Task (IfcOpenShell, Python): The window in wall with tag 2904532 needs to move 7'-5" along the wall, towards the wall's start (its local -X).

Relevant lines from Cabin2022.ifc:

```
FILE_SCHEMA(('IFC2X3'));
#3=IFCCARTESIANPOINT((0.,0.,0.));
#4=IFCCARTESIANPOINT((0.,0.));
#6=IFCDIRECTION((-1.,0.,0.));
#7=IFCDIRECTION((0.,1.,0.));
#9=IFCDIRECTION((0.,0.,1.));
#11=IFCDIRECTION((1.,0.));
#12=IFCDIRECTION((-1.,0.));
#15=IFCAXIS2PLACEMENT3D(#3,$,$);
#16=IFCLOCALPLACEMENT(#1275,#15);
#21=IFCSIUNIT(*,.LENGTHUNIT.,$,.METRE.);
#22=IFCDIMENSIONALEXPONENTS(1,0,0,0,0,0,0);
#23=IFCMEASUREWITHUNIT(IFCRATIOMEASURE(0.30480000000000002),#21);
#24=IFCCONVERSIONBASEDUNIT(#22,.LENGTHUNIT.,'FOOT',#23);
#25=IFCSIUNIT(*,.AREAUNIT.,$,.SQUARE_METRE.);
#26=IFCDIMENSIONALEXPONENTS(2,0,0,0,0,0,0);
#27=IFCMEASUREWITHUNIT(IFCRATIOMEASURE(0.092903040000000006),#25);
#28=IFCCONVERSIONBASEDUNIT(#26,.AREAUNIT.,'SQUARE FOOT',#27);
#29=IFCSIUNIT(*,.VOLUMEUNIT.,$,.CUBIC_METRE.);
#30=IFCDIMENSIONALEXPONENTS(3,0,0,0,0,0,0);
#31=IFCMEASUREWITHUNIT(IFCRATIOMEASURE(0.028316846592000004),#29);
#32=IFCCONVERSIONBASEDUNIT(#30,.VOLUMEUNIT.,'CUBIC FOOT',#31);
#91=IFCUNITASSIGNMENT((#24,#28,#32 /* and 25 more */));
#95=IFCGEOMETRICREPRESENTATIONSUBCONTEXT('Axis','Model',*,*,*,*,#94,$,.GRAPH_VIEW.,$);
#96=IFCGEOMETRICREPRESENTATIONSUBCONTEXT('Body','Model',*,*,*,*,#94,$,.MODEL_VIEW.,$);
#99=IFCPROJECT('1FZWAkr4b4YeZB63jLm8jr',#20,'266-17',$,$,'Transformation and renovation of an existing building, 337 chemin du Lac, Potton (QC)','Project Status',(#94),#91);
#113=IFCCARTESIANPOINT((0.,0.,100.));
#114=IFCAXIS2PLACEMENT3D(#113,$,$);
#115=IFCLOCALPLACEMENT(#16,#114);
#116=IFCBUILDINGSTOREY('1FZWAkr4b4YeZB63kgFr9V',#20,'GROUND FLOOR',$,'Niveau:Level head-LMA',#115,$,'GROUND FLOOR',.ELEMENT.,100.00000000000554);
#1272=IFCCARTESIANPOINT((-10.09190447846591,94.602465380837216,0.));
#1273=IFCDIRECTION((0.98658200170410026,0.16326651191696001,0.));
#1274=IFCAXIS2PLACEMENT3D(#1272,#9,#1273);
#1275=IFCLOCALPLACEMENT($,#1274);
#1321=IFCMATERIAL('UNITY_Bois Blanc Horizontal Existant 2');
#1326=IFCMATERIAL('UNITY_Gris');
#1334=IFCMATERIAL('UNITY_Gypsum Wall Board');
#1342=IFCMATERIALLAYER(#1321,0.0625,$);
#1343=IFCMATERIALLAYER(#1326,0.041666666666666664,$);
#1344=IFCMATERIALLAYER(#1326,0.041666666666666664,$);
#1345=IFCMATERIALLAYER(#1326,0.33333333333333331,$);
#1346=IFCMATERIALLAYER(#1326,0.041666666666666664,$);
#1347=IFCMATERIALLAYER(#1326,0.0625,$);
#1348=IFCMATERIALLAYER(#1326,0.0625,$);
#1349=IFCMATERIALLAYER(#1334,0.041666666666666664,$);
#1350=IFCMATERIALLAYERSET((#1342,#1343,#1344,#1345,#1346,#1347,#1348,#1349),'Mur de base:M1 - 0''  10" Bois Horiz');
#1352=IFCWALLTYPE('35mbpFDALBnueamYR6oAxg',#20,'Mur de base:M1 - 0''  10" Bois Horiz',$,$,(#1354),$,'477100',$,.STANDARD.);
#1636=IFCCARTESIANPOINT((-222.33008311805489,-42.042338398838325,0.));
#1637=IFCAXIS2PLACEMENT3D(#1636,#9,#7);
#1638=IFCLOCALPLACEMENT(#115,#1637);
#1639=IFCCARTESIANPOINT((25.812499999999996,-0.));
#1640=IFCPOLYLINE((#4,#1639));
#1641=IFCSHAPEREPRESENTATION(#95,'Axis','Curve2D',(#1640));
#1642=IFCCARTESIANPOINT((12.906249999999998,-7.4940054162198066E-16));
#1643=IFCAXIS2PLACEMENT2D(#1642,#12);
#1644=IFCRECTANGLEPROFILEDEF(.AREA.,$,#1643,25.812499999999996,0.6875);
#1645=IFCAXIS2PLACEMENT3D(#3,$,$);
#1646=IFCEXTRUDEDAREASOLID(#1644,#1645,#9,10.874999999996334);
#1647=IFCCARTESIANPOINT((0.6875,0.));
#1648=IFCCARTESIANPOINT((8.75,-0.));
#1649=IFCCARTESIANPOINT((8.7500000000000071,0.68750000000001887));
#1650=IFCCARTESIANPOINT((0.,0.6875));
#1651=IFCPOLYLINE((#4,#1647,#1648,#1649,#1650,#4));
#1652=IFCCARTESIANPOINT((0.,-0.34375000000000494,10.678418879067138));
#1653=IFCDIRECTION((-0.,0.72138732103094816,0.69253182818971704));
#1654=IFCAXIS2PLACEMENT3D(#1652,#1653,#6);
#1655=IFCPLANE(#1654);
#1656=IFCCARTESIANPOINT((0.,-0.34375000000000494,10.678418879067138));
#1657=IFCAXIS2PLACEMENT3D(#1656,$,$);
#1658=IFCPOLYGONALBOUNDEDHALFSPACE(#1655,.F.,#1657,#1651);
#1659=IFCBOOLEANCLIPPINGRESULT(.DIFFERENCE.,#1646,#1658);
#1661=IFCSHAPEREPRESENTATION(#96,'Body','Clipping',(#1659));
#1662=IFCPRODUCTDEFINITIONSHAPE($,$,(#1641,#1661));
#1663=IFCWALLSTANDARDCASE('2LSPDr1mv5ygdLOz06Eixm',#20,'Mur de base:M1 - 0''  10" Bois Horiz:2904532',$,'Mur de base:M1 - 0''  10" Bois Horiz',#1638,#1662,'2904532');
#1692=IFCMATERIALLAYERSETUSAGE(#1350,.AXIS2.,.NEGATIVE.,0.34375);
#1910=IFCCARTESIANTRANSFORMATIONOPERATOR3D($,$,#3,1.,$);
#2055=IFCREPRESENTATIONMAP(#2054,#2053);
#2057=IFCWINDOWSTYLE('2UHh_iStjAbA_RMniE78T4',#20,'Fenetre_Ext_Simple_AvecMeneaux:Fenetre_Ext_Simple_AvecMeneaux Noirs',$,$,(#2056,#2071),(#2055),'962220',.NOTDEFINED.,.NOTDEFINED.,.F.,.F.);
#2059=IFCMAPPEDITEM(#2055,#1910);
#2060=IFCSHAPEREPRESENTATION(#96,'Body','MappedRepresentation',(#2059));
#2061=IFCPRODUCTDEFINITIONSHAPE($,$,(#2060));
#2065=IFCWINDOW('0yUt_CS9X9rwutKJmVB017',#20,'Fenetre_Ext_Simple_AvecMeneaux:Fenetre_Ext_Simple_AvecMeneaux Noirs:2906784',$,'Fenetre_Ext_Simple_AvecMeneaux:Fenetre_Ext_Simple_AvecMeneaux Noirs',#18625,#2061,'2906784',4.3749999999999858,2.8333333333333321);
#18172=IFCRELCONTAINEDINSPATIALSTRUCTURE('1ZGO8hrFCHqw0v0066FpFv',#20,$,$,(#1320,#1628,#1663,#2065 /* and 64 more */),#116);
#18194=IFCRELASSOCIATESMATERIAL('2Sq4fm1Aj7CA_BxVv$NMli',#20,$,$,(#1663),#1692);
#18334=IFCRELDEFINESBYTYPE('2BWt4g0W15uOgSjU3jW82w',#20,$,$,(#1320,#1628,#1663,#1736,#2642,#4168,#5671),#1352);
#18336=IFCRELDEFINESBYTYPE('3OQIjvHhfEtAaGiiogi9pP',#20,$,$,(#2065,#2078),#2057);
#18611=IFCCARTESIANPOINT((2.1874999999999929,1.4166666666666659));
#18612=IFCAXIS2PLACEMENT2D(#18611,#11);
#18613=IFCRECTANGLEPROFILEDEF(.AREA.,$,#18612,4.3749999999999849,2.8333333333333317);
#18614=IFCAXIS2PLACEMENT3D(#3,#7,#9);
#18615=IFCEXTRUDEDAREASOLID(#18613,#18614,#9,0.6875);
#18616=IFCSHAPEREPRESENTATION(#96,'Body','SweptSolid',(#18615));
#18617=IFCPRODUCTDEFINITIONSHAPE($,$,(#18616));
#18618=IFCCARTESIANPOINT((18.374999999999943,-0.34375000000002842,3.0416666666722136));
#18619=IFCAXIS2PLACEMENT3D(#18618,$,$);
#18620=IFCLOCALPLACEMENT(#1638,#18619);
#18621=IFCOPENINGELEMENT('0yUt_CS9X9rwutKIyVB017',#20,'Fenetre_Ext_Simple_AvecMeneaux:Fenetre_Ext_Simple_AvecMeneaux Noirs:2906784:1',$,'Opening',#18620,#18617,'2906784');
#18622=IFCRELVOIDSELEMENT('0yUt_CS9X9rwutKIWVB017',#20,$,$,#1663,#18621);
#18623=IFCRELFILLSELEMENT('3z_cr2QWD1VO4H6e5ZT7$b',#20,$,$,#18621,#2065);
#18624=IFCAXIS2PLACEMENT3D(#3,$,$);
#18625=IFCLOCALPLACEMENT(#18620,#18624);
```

```python
import ifcopenshell
import ifcopenshell.api.geometry
import ifcopenshell.util.placement
import ifcopenshell.util.unit

model = ifcopenshell.open("Cabin2022.ifc")
unit_scale = ifcopenshell.util.unit.calculate_unit_scale(model)

window = model.by_guid("0yUt_CS9X9rwutKJmVB017")
opening = window.FillsVoids[0].RelatingOpeningElement
wall = opening.VoidsElements[0].RelatingBuildingElement

wall_matrix = ifcopenshell.util.placement.get_local_placement(wall.ObjectPlacement)
shift = wall_matrix[:3, 0] * -89 * 0.0254 / unit_scale
before = ifcopenshell.util.placement.get_local_placement(window.ObjectPlacement)[:3, 3].copy()

# The window is placed relative to its opening, so it follows when the opening moves.
matrix = ifcopenshell.util.placement.get_local_placement(opening.ObjectPlacement)
matrix[:3, 3] += shift
ifcopenshell.api.geometry.edit_object_placement(
    model, product=opening, matrix=matrix, is_si=False, should_transform_children=True
)

after = ifcopenshell.util.placement.get_local_placement(window.ObjectPlacement)[:3, 3]
print("window moved by", (after - before).round(3) + 0.0)

model.write("Cabin2022-out.ifc")
```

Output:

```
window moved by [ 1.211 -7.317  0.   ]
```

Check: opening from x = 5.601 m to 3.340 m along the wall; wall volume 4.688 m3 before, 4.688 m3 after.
